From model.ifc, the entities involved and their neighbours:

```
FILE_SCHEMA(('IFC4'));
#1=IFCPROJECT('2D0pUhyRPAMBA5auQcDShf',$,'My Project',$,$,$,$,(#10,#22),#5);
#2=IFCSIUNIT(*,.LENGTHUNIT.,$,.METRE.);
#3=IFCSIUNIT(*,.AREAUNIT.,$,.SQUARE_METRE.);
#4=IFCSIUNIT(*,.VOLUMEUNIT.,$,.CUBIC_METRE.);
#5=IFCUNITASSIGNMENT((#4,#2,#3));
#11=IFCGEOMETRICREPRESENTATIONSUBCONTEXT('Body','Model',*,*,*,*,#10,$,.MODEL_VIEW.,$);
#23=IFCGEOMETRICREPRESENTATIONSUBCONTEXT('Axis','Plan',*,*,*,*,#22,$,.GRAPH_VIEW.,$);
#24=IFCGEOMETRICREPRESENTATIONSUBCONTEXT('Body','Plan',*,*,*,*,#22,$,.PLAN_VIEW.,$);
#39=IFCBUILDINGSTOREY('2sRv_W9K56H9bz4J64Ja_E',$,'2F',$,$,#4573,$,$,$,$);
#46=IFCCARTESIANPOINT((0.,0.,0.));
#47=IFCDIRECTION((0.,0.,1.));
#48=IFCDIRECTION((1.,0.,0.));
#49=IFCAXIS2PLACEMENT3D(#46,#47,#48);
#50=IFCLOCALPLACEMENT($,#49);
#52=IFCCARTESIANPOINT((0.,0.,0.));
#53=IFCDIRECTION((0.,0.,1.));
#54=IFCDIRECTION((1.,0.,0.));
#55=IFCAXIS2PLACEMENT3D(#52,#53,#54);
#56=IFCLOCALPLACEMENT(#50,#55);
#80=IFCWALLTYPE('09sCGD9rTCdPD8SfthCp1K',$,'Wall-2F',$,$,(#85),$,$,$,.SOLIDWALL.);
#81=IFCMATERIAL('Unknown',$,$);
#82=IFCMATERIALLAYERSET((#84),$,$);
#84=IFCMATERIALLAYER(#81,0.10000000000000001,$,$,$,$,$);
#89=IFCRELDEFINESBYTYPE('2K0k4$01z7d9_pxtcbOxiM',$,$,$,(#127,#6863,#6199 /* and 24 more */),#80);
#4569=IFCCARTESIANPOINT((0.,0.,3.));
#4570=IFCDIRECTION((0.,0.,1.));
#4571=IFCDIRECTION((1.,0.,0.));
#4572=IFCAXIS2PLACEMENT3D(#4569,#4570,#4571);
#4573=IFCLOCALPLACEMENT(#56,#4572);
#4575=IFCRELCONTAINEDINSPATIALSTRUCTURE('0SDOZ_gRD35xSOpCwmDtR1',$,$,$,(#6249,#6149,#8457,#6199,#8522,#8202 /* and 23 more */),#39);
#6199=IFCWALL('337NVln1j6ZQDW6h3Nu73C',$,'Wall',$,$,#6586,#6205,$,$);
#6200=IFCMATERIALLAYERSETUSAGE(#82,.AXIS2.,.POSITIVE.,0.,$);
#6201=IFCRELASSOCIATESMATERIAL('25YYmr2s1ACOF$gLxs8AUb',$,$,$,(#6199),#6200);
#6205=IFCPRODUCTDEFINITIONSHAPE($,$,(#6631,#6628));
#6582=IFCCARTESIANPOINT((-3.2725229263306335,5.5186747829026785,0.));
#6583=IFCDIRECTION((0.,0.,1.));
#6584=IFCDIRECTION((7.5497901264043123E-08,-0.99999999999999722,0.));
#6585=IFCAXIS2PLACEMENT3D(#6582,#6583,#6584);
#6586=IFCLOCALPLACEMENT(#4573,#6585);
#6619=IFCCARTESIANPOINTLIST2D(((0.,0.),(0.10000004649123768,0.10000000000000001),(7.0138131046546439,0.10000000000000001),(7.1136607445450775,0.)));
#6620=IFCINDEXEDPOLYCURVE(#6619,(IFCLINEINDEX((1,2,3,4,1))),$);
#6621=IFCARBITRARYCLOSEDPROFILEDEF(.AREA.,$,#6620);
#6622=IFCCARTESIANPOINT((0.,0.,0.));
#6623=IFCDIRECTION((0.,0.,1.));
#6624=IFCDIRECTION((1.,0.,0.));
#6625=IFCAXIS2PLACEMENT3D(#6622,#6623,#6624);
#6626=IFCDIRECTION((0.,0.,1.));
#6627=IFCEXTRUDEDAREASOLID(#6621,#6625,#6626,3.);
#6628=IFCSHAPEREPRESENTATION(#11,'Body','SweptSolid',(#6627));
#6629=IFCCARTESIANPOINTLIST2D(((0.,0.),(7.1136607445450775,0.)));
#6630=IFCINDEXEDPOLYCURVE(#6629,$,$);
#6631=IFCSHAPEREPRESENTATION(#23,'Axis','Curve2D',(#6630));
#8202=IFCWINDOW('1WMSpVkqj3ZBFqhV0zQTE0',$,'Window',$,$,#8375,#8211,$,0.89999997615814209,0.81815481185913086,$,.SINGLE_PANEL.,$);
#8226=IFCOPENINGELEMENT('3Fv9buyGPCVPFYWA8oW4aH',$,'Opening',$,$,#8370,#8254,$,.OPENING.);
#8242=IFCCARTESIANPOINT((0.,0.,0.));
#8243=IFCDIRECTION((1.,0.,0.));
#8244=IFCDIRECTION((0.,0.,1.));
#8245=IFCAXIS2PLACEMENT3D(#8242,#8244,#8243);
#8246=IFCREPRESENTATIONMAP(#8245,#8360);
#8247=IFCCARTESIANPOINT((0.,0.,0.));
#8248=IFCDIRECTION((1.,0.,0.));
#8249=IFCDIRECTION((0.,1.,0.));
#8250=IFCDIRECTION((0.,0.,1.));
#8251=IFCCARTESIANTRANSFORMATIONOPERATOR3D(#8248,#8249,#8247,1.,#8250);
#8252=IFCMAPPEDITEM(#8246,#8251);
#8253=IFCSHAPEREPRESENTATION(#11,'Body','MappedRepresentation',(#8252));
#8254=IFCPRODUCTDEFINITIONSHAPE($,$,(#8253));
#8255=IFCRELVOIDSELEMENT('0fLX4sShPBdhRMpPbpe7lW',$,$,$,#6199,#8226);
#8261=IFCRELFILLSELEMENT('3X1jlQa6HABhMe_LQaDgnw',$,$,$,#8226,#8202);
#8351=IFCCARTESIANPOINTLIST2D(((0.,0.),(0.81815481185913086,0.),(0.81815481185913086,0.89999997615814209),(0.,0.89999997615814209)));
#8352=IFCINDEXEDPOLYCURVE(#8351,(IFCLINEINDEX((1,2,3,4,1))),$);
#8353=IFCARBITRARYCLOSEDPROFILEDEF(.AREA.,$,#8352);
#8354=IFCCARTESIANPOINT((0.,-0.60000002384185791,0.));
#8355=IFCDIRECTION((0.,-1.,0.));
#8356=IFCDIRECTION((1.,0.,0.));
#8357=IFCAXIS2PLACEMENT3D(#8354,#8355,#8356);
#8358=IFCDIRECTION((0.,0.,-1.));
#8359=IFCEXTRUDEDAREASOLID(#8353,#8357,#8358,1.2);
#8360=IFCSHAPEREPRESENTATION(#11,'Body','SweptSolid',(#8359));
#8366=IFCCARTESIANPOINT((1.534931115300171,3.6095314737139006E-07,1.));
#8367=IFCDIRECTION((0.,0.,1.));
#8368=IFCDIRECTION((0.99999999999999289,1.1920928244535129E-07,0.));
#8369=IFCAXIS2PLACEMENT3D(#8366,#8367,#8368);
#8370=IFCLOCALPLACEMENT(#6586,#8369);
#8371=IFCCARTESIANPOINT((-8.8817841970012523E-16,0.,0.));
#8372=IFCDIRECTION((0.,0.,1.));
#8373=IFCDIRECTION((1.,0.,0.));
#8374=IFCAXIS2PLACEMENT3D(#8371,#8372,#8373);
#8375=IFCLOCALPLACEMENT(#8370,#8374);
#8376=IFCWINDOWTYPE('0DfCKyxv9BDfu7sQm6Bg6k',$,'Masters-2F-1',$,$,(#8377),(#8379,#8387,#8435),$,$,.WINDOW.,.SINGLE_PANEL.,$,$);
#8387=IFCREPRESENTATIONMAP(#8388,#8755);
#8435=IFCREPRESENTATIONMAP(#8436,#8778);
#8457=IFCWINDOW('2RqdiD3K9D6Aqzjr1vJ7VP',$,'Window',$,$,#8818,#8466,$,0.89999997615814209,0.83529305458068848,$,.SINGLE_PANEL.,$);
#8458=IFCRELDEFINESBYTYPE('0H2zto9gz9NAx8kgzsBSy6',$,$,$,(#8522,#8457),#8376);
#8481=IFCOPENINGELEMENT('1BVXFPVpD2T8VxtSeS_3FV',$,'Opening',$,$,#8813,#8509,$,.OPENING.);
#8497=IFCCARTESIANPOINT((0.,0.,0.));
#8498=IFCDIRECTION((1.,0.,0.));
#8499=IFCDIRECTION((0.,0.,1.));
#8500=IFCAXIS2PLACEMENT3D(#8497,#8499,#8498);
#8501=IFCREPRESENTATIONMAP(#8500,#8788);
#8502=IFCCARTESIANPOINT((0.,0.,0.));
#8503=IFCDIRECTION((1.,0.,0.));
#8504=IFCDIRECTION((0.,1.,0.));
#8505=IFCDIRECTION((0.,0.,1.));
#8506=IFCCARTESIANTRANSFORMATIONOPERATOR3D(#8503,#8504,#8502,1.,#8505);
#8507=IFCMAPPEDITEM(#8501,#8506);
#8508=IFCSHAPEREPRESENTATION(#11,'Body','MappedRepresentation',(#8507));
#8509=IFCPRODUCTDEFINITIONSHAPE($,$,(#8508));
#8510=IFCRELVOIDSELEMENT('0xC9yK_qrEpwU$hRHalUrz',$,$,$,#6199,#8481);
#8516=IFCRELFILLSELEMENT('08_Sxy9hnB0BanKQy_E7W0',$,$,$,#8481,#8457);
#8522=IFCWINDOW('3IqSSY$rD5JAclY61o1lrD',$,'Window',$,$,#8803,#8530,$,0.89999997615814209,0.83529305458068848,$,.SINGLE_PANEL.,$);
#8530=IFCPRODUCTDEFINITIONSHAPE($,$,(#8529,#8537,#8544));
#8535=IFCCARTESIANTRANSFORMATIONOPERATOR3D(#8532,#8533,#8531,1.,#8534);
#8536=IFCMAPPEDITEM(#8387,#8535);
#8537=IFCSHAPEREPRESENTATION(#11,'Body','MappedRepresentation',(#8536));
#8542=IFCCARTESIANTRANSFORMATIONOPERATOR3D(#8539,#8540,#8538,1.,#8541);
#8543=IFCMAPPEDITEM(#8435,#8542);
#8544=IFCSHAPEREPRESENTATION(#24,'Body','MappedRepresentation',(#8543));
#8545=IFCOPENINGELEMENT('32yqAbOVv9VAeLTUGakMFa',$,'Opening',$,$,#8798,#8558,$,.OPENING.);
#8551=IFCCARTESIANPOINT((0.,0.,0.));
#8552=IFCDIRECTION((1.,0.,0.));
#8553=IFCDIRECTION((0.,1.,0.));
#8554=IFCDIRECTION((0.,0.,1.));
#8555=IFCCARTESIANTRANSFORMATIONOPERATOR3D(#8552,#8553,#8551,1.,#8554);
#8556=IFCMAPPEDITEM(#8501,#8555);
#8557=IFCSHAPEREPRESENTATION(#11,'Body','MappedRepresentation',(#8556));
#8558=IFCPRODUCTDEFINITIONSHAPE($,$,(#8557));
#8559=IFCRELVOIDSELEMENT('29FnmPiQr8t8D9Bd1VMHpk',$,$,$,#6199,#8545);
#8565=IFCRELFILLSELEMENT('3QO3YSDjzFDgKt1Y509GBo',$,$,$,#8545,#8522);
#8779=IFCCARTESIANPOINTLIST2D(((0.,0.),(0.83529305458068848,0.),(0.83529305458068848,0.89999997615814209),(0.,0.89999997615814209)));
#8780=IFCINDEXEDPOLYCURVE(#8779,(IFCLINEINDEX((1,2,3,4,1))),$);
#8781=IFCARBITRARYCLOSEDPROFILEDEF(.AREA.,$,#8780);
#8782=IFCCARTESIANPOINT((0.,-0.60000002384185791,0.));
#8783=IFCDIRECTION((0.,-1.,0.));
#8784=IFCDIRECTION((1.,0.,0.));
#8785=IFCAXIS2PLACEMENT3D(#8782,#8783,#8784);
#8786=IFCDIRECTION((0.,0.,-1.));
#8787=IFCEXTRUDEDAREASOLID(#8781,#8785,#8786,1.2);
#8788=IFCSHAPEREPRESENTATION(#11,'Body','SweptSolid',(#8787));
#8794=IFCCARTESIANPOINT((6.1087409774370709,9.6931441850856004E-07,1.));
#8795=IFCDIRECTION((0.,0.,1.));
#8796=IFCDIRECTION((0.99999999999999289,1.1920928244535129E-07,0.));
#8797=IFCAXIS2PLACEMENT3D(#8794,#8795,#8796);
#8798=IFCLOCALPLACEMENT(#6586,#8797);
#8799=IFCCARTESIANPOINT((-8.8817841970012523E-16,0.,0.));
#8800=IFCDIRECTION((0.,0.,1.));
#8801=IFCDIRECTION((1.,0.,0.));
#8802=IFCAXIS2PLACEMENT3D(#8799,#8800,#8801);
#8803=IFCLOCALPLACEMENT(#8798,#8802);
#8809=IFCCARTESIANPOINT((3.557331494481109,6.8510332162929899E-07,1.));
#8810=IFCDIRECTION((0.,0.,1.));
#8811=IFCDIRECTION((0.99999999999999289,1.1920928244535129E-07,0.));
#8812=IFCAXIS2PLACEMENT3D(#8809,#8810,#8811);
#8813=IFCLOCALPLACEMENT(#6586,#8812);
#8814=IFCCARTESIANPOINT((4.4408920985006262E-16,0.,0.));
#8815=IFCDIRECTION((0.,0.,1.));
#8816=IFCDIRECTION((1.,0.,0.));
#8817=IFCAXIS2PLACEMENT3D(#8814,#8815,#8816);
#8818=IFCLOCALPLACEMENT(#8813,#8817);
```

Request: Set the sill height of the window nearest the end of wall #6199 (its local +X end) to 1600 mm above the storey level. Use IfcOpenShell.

```python
import numpy as np
import ifcopenshell
import ifcopenshell.api.geometry
import ifcopenshell.geom
import ifcopenshell.util.element
import ifcopenshell.util.placement
import ifcopenshell.util.shape
import ifcopenshell.util.unit

model = ifcopenshell.open("model.ifc")
unit_scale = ifcopenshell.util.unit.calculate_unit_scale(model)

window = model.by_guid("3IqSSY$rD5JAclY61o1lrD")
opening = window.FillsVoids[0].RelatingOpeningElement
storey = ifcopenshell.util.element.get_container(window, ifc_class="IfcBuildingStorey")
level = ifcopenshell.util.placement.get_local_placement(storey.ObjectPlacement)[2, 3]

# The opening's origin need not be at the sill, so measure its lowest point.
shape = ifcopenshell.geom.create_shape(ifcopenshell.geom.settings(), opening)
bottom = ifcopenshell.util.shape.get_shape_bottom_elevation(shape, shape.geometry) / unit_scale
dz = level + 1.6 / unit_scale - bottom

shift = np.array([0.0, 0.0, dz])
# The window is placed relative to its opening, so it follows when the opening moves.
matrix = ifcopenshell.util.placement.get_local_placement(opening.ObjectPlacement)
matrix[:3, 3] += shift
ifcopenshell.api.geometry.edit_object_placement(
    model, product=opening, matrix=matrix, is_si=False, should_transform_children=True
)

print(f"moved by {dz * unit_scale:+.3f} m")

model.write("model_v2.ifc")
```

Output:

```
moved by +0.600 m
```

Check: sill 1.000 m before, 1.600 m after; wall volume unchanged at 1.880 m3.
